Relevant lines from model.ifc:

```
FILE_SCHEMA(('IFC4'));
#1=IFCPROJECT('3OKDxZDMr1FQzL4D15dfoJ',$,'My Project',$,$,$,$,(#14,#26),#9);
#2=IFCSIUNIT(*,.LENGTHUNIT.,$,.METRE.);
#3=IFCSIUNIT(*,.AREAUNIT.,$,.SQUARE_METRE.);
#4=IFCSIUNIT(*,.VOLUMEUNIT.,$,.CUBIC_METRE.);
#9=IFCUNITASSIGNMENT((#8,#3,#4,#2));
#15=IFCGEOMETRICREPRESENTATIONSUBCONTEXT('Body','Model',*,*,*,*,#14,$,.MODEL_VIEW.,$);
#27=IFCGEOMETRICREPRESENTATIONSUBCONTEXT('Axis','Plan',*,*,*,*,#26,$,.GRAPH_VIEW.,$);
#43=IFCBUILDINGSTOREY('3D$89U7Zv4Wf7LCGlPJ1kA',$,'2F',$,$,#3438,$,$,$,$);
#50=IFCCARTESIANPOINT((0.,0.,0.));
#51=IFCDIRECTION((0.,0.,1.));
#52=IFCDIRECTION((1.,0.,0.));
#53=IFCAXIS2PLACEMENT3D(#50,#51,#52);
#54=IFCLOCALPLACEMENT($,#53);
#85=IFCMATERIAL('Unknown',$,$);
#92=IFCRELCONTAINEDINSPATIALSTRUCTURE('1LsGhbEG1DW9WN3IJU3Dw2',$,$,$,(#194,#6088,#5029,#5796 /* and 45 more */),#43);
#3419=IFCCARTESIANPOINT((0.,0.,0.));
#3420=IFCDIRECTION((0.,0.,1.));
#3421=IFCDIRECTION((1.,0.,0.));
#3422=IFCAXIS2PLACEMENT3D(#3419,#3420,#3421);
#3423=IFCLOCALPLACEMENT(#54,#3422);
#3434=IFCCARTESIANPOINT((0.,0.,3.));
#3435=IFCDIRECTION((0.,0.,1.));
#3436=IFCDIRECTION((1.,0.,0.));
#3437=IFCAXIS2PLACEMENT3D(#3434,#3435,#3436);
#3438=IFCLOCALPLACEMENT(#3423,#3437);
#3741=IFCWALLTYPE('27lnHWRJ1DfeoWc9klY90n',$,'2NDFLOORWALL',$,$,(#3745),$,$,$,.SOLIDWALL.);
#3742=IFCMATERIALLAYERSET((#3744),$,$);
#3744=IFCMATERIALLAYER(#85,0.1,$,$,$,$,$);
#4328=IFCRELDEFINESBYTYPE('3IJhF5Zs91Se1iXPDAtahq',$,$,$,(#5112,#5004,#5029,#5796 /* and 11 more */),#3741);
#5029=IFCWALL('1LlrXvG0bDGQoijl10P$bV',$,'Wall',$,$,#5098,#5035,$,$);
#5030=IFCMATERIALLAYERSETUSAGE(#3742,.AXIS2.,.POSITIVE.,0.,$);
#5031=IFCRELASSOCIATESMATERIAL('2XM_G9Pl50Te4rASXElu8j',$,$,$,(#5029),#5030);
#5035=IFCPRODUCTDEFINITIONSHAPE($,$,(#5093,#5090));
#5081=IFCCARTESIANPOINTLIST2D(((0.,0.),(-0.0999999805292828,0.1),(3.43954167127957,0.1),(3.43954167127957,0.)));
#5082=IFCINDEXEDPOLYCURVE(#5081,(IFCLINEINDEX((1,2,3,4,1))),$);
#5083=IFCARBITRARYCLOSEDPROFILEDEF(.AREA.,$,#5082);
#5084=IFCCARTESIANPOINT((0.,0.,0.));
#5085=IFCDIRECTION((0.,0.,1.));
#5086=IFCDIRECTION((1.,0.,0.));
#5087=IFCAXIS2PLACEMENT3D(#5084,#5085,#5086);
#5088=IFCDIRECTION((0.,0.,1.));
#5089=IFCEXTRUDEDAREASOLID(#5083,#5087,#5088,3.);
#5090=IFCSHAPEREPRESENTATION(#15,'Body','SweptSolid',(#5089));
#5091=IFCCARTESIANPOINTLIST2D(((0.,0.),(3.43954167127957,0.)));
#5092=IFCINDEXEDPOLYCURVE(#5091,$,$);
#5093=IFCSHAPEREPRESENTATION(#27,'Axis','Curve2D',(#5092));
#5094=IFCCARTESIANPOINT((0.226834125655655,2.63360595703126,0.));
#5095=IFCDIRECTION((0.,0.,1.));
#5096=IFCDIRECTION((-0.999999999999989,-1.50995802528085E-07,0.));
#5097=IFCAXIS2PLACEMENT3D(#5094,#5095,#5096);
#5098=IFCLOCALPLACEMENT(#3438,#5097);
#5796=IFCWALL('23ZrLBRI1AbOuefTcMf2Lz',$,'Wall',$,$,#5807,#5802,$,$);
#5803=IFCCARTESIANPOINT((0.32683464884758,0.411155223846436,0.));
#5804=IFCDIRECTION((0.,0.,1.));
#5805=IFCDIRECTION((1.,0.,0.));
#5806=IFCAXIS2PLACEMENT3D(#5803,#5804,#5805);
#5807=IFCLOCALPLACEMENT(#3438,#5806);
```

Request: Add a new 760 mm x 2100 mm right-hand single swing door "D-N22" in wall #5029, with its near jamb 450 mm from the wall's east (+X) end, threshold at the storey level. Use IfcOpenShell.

```python
import numpy as np
import ifcopenshell
import ifcopenshell.api.feature
import ifcopenshell.api.geometry
import ifcopenshell.api.root
import ifcopenshell.api.spatial
import ifcopenshell.geom
import ifcopenshell.util.element
import ifcopenshell.util.placement
import ifcopenshell.util.representation
import ifcopenshell.util.shape
import ifcopenshell.util.unit

model = ifcopenshell.open("model.ifc")
unit_scale = ifcopenshell.util.unit.calculate_unit_scale(model)
settings = ifcopenshell.geom.settings()


def volume(element):
    """Net volume in cubic metres, openings subtracted."""
    shape = ifcopenshell.geom.create_shape(settings, element)
    return ifcopenshell.util.shape.get_volume(shape.geometry)


wall = model.by_guid("1LlrXvG0bDGQoijl10P$bV")
storey = ifcopenshell.util.element.get_container(wall, ifc_class="IfcBuildingStorey")
context = ifcopenshell.util.representation.get_context(model, "Model", "Body", "MODEL_VIEW")
before = volume(wall)

width, height, from_end, sill = 0.76, 2.1, 0.45, 0.0  # metres

# The wall runs along its own X axis, and the end named is its -X end.
wall_shape = ifcopenshell.geom.create_shape(settings, wall)
x, y, z = ifcopenshell.util.shape.get_vertices(wall_shape.geometry).T
start = x.min() + from_end
face, thickness = float(y.min()), float(y.max() - y.min())
wall_matrix = ifcopenshell.util.placement.get_local_placement(wall.ObjectPlacement)
level = ifcopenshell.util.placement.get_local_placement(storey.ObjectPlacement)[2, 3]


def in_wall(x, y):
    """Placement at x, y metres in the wall's axes, at sill height."""
    matrix = wall_matrix.copy()
    matrix[:, 3] = wall_matrix @ np.array([x / unit_scale, y / unit_scale, 0.0, 1.0])
    matrix[2, 3] = level + sill / unit_scale
    return matrix


# Opening: a box that overshoots both wall faces by 50 mm.
opening = ifcopenshell.api.root.create_entity(model, ifc_class="IfcOpeningElement", predefined_type="OPENING")
box = ifcopenshell.api.geometry.add_wall_representation(
    model, context=context, length=width, height=height, thickness=thickness + 0.1
)
ifcopenshell.api.geometry.assign_representation(model, product=opening, representation=box)
ifcopenshell.api.geometry.edit_object_placement(model, product=opening, matrix=in_wall(start, face - 0.05), is_si=False)
ifcopenshell.api.feature.add_feature(model, feature=opening, element=wall)

door = ifcopenshell.api.root.create_entity(model, ifc_class="IfcDoor", name="D-N22", predefined_type="DOOR")
door.OverallWidth, door.OverallHeight = width / unit_scale, height / unit_scale
door.OperationType = "SINGLE_SWING_RIGHT"
body = ifcopenshell.api.geometry.add_door_representation(
    model,
    context=context,
    overall_width=door.OverallWidth,
    overall_height=door.OverallHeight,
    operation_type="SINGLE_SWING_RIGHT",
    lining_properties={"LiningDepth": thickness / unit_scale, "ThresholdDepth": thickness / unit_scale},
)
ifcopenshell.api.geometry.assign_representation(model, product=door, representation=body)
ifcopenshell.api.spatial.assign_container(model, products=[door], relating_structure=storey)
ifcopenshell.api.feature.add_filling(model, opening=opening, element=door)

# The lining spans the wall, so the door starts at the wall face.
ifcopenshell.api.geometry.edit_object_placement(model, product=door, matrix=in_wall(start, face), is_si=False)

after = volume(wall)

print(f"wall volume {before:.3f} -> {after:.3f} m3")

model.write("model_v2.ifc")
```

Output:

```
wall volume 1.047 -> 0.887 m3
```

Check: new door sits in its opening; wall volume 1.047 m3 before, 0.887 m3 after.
